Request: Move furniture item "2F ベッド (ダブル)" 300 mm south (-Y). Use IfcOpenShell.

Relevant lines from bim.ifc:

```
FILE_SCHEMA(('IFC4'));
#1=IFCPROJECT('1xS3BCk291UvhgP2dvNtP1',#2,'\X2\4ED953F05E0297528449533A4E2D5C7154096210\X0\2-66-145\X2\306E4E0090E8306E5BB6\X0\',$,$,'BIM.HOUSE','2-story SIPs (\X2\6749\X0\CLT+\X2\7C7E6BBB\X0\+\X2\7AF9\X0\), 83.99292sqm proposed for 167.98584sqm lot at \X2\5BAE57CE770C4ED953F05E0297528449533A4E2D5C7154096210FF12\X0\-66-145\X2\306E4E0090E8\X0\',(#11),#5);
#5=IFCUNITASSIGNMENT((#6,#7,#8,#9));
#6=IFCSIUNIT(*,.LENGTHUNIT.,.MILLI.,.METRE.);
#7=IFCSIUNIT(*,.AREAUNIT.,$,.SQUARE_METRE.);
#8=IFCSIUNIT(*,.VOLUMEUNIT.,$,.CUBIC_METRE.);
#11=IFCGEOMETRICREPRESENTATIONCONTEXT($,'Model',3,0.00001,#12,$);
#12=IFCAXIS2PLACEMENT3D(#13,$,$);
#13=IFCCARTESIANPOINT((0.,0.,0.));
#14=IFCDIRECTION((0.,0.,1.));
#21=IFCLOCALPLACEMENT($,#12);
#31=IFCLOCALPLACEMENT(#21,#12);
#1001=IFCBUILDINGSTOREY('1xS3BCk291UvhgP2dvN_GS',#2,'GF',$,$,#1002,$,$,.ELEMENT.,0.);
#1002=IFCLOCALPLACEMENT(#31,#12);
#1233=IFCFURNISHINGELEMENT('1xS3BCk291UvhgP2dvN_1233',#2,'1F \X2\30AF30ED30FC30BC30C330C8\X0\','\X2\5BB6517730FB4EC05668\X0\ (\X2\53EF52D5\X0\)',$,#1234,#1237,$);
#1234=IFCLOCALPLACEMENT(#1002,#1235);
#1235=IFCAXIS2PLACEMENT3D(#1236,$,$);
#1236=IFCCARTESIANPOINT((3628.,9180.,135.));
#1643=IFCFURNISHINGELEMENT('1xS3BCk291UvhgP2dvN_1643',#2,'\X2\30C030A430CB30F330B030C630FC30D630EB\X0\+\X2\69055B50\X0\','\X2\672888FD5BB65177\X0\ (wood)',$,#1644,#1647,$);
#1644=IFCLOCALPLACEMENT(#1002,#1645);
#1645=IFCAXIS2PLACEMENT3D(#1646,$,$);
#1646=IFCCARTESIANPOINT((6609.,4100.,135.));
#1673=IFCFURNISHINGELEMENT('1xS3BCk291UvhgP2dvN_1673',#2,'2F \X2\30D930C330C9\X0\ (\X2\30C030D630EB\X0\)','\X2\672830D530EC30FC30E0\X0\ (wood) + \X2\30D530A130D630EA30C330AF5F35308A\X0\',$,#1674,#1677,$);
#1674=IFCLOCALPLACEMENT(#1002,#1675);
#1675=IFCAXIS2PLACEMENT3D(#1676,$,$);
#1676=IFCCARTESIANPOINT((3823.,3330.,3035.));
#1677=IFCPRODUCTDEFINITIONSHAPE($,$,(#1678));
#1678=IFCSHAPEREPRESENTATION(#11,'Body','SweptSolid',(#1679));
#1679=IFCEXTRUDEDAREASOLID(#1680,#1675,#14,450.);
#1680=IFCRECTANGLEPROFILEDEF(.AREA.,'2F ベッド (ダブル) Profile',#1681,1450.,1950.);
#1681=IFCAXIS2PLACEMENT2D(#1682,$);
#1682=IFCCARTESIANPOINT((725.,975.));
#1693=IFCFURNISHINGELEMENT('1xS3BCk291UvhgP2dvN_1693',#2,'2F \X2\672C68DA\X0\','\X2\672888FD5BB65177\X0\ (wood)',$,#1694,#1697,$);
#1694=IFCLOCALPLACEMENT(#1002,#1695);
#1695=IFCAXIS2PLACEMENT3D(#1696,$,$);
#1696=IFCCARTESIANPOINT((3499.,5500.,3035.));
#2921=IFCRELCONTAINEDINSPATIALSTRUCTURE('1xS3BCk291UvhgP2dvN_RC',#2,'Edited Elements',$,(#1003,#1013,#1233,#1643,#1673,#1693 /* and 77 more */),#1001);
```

```python
import ifcopenshell
import ifcopenshell.api.geometry
import ifcopenshell.util.placement
import ifcopenshell.util.unit

model = ifcopenshell.open("bim.ifc")
unit_scale = ifcopenshell.util.unit.calculate_unit_scale(model)

item = model.by_guid("1xS3BCk291UvhgP2dvN_1673")
matrix = ifcopenshell.util.placement.get_local_placement(item.ObjectPlacement)
matrix[1, 3] -= 0.3 / unit_scale
ifcopenshell.api.geometry.edit_object_placement(model, product=item, matrix=matrix, is_si=False)

print(ifcopenshell.util.placement.get_local_placement(item.ObjectPlacement).round(3) + 0.0)

model.write("bim-out.ifc")
```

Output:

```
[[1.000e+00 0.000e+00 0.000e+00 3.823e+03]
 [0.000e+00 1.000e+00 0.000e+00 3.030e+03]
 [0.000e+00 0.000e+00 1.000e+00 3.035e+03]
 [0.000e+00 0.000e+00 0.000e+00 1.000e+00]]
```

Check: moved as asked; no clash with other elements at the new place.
